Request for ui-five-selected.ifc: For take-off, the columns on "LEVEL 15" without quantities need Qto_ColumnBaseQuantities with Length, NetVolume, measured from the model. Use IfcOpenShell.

First a look at what the model holds.

```python
import ifcopenshell
import ifcopenshell.util.element
import ifcopenshell.util.unit

model = ifcopenshell.open("ui-five-selected.ifc")
print(model.schema)
for unit_type in ("LENGTHUNIT", "AREAUNIT", "VOLUMEUNIT"):
    print(unit_type, ifcopenshell.util.unit.calculate_unit_scale(model, unit_type))
storey = next(s for s in model.by_type("IfcBuildingStorey") if s.Name == "LEVEL 15")
columns = [e for e in ifcopenshell.util.element.get_decomposition(storey) if e.is_a("IfcColumn")]
for e in sorted(columns, key=lambda e: e.id()):
    print(e.id(), e.is_a(), e.Name, list(ifcopenshell.util.element.get_psets(e, qtos_only=True)), sep=" | ")
```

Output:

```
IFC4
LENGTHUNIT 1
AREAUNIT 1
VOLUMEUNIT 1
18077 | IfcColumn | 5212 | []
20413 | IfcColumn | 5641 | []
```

```python
import ifcopenshell
import ifcopenshell.api.pset
import ifcopenshell.geom
import ifcopenshell.util.element
import ifcopenshell.util.shape
import ifcopenshell.util.unit

model = ifcopenshell.open("ui-five-selected.ifc")
unit_scale = ifcopenshell.util.unit.calculate_unit_scale(model)
volume_scale = ifcopenshell.util.unit.calculate_unit_scale(model, "VOLUMEUNIT")
settings = ifcopenshell.geom.settings()

storey = next(s for s in model.by_type("IfcBuildingStorey") if s.Name == "LEVEL 15")
columns = [e for e in ifcopenshell.util.element.get_decomposition(storey) if e.is_a("IfcColumn")]

for e in sorted(columns, key=lambda e: e.id()):
    if ifcopenshell.util.element.get_psets(e, qtos_only=True, should_inherit=False):
        continue
    # Geometry comes back in metres, in the element's own axes.
    shape = ifcopenshell.geom.create_shape(settings, e)
    values = {
        "Length": ifcopenshell.util.shape.get_z(shape.geometry) / unit_scale,
        "NetVolume": ifcopenshell.util.shape.get_volume(shape.geometry) / volume_scale,
    }
    qto = ifcopenshell.api.pset.add_qto(model, product=e, name="Qto_ColumnBaseQuantities")
    ifcopenshell.api.pset.edit_qto(model, qto=qto, properties=values)
    print(e.id(), {k: round(v, 3) for k, v in values.items()})

model.write("ui-five-selected_updated.ifc")
```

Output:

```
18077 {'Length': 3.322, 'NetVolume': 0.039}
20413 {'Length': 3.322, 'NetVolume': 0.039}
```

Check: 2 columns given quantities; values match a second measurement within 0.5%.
